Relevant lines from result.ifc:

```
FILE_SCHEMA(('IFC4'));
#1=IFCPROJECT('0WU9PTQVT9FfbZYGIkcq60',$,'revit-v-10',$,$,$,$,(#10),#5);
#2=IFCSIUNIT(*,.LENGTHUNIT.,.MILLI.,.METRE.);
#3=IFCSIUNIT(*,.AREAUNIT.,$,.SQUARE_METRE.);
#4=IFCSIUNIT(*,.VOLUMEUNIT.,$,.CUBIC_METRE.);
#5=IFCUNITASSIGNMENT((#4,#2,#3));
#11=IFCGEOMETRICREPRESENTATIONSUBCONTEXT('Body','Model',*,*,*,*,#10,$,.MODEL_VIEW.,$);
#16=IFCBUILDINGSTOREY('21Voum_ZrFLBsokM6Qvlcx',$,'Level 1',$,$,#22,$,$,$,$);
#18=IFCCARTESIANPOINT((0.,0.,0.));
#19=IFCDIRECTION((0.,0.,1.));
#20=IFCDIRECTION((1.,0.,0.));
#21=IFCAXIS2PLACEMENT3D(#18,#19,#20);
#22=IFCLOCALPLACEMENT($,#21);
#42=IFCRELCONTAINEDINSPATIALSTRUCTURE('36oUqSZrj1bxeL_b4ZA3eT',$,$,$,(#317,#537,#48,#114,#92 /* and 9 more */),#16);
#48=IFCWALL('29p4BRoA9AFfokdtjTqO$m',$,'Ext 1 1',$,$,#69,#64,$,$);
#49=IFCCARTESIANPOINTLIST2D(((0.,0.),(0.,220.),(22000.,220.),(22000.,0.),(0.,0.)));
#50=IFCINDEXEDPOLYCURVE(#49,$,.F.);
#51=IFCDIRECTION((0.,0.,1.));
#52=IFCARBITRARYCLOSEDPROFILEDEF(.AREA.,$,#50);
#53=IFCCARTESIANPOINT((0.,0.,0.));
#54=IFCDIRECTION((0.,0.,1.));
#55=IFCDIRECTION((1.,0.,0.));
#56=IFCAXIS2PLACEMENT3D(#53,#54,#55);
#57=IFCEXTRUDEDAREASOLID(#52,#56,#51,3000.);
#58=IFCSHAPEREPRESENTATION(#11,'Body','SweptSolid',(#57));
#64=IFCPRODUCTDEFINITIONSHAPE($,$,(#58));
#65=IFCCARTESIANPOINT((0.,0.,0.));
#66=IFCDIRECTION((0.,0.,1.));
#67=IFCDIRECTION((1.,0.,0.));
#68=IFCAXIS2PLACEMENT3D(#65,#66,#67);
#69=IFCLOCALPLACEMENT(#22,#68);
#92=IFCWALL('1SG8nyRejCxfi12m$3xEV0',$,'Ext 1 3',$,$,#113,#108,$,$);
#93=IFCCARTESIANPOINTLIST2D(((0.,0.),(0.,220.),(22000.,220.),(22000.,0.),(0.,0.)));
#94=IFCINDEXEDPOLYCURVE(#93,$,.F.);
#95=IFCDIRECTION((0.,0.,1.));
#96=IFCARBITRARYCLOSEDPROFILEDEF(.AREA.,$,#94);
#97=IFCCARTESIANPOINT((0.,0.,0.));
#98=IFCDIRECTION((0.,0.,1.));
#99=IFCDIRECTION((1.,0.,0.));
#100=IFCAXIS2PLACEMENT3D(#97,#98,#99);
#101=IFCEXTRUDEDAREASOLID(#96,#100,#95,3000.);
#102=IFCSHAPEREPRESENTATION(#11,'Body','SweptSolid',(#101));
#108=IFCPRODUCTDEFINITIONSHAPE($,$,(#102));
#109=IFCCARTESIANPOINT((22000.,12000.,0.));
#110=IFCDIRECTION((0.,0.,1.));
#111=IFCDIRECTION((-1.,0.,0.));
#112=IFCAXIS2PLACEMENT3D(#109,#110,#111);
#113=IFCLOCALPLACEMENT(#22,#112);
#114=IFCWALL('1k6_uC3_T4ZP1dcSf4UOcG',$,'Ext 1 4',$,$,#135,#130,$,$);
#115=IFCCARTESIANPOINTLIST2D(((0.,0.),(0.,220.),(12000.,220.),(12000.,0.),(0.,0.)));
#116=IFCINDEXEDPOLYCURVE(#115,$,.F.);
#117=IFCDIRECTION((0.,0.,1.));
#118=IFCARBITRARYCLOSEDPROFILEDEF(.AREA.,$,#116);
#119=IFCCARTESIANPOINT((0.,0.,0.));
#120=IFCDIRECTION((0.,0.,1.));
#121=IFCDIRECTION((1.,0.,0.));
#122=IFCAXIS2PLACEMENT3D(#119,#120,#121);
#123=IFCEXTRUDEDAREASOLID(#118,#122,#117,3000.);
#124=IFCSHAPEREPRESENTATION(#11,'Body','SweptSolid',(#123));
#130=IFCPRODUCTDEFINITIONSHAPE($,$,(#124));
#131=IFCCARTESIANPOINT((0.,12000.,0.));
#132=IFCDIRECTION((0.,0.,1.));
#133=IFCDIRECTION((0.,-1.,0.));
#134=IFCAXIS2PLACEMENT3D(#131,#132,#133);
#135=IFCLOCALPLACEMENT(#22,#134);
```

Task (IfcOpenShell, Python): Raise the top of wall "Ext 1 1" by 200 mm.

```python
import ifcopenshell
import ifcopenshell.geom
import ifcopenshell.util.representation
import ifcopenshell.util.shape
import ifcopenshell.util.unit

model = ifcopenshell.open("result.ifc")
unit_scale = ifcopenshell.util.unit.calculate_unit_scale(model)
settings = ifcopenshell.geom.settings()


def volume(element):
    """Net volume in cubic metres, openings subtracted."""
    shape = ifcopenshell.geom.create_shape(settings, element)
    return ifcopenshell.util.shape.get_volume(shape.geometry)


wall = model.by_guid("29p4BRoA9AFfokdtjTqO$m")
before = volume(wall)

body = ifcopenshell.util.representation.get_representation(wall, "Model", "Body")
solid = body.Items[0]
old_height = solid.Depth
solid.Depth += 0.2 / unit_scale
after = volume(wall)

print(f"height {old_height:g} -> {solid.Depth:g}, volume {before:.3f} -> {after:.3f} m3")

model.write("result_v2.ifc")
```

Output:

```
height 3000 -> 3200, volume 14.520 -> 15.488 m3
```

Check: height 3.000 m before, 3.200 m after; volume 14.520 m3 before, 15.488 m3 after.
